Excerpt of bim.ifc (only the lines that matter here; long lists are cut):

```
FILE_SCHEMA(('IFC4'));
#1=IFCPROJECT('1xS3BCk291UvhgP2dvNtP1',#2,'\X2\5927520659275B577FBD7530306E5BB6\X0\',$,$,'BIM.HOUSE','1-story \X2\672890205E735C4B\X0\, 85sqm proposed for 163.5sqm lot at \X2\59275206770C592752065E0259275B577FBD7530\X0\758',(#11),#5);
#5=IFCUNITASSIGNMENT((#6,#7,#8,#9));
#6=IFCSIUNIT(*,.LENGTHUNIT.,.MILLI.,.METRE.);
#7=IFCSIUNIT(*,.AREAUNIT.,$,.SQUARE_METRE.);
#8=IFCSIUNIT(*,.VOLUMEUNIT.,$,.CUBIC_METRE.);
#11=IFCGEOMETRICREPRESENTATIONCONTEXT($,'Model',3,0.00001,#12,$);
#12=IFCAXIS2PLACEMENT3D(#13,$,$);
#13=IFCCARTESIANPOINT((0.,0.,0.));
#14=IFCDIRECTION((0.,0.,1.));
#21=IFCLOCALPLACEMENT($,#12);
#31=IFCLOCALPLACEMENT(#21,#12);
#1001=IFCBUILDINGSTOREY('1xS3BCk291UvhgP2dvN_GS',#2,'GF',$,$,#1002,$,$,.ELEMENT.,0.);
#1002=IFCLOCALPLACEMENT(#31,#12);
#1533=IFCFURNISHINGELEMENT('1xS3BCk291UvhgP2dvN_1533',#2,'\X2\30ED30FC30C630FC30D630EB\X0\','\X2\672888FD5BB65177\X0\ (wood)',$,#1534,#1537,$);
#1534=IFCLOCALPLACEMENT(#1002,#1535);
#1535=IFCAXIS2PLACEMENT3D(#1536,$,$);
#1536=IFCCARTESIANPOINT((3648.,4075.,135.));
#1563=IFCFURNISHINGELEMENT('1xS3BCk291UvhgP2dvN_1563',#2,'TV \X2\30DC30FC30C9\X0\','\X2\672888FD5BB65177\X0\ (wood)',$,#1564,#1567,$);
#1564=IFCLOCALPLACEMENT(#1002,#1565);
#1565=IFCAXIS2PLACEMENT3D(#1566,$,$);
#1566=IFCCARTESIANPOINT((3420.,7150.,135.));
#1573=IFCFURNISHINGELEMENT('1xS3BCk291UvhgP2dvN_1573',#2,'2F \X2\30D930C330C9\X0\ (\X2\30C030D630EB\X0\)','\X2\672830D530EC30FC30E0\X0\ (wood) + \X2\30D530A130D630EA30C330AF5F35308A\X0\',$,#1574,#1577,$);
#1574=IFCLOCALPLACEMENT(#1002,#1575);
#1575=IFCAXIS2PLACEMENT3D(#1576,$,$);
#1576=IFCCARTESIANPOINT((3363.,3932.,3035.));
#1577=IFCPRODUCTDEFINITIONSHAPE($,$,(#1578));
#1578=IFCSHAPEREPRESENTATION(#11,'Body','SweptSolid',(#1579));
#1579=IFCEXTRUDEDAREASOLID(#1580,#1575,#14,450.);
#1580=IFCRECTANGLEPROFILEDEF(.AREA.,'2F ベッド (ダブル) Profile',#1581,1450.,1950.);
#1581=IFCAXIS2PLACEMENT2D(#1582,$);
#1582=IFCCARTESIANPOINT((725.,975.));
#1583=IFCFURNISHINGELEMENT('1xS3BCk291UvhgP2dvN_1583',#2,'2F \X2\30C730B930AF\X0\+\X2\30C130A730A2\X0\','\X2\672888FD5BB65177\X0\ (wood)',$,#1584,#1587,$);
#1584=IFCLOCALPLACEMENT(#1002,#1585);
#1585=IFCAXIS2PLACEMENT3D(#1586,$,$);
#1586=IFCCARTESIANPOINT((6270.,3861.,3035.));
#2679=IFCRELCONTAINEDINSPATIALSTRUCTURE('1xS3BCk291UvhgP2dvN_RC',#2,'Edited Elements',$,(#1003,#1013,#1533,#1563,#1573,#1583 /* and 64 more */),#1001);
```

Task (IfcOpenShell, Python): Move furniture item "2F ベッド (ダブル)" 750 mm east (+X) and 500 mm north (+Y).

```python
import ifcopenshell
import ifcopenshell.api.geometry
import ifcopenshell.util.placement
import ifcopenshell.util.unit

model = ifcopenshell.open("bim.ifc")
unit_scale = ifcopenshell.util.unit.calculate_unit_scale(model)

item = model.by_id(1573)
matrix = ifcopenshell.util.placement.get_local_placement(item.ObjectPlacement)
matrix[0, 3] += 0.75 / unit_scale
matrix[1, 3] += 0.5 / unit_scale
ifcopenshell.api.geometry.edit_object_placement(model, product=item, matrix=matrix, is_si=False)

print(ifcopenshell.util.placement.get_local_placement(item.ObjectPlacement).round(3) + 0.0)

model.write("bim-out.ifc")
```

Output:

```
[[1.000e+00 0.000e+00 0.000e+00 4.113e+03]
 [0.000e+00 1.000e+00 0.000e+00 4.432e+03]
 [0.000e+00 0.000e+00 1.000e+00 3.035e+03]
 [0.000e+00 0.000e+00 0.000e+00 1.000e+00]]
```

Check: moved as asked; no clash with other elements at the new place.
